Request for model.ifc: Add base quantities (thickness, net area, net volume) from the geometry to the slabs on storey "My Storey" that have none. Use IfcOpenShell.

First a look at what the model holds.

```python
import ifcopenshell
import ifcopenshell.util.element
import ifcopenshell.util.unit

model = ifcopenshell.open("model.ifc")
print(model.schema)
for unit_type in ("LENGTHUNIT", "AREAUNIT", "VOLUMEUNIT"):
    print(unit_type, ifcopenshell.util.unit.calculate_unit_scale(model, unit_type))
storey = next(s for s in model.by_type("IfcBuildingStorey") if s.Name == "My Storey")
slabs = [e for e in ifcopenshell.util.element.get_decomposition(storey) if e.is_a("IfcSlab")]
for e in sorted(slabs, key=lambda e: e.id()):
    print(e.id(), e.is_a(), e.Name, list(ifcopenshell.util.element.get_psets(e, qtos_only=True)), sep=" | ")
```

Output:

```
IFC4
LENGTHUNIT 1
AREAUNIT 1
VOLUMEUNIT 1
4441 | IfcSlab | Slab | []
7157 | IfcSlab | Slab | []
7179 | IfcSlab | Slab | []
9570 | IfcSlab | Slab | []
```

```python
import ifcopenshell
import ifcopenshell.api.pset
import ifcopenshell.geom
import ifcopenshell.util.element
import ifcopenshell.util.shape
import ifcopenshell.util.unit

model = ifcopenshell.open("model.ifc")
unit_scale = ifcopenshell.util.unit.calculate_unit_scale(model)
area_scale = ifcopenshell.util.unit.calculate_unit_scale(model, "AREAUNIT")
volume_scale = ifcopenshell.util.unit.calculate_unit_scale(model, "VOLUMEUNIT")
settings = ifcopenshell.geom.settings()

storey = next(s for s in model.by_type("IfcBuildingStorey") if s.Name == "My Storey")
slabs = [e for e in ifcopenshell.util.element.get_decomposition(storey) if e.is_a("IfcSlab")]

for e in sorted(slabs, key=lambda e: e.id()):
    if ifcopenshell.util.element.get_psets(e, qtos_only=True, should_inherit=False):
        continue
    # Geometry comes back in metres, in the element's own axes.
    shape = ifcopenshell.geom.create_shape(settings, e)
    values = {
        "Width": ifcopenshell.util.shape.get_z(shape.geometry) / unit_scale,
        "NetArea": ifcopenshell.util.shape.get_footprint_area(shape.geometry) / area_scale,
        "NetVolume": ifcopenshell.util.shape.get_volume(shape.geometry) / volume_scale,
    }
    qto = ifcopenshell.api.pset.add_qto(model, product=e, name="Qto_SlabBaseQuantities")
    ifcopenshell.api.pset.edit_qto(model, qto=qto, properties=values)
    print(e.id(), {k: round(v, 3) for k, v in values.items()})

model.write("model_v2.ifc")
```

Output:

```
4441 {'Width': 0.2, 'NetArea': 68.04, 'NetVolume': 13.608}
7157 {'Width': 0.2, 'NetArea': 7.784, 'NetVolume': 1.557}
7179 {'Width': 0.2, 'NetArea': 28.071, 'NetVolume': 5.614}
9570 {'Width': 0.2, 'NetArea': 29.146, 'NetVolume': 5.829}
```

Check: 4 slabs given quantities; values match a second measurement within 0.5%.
